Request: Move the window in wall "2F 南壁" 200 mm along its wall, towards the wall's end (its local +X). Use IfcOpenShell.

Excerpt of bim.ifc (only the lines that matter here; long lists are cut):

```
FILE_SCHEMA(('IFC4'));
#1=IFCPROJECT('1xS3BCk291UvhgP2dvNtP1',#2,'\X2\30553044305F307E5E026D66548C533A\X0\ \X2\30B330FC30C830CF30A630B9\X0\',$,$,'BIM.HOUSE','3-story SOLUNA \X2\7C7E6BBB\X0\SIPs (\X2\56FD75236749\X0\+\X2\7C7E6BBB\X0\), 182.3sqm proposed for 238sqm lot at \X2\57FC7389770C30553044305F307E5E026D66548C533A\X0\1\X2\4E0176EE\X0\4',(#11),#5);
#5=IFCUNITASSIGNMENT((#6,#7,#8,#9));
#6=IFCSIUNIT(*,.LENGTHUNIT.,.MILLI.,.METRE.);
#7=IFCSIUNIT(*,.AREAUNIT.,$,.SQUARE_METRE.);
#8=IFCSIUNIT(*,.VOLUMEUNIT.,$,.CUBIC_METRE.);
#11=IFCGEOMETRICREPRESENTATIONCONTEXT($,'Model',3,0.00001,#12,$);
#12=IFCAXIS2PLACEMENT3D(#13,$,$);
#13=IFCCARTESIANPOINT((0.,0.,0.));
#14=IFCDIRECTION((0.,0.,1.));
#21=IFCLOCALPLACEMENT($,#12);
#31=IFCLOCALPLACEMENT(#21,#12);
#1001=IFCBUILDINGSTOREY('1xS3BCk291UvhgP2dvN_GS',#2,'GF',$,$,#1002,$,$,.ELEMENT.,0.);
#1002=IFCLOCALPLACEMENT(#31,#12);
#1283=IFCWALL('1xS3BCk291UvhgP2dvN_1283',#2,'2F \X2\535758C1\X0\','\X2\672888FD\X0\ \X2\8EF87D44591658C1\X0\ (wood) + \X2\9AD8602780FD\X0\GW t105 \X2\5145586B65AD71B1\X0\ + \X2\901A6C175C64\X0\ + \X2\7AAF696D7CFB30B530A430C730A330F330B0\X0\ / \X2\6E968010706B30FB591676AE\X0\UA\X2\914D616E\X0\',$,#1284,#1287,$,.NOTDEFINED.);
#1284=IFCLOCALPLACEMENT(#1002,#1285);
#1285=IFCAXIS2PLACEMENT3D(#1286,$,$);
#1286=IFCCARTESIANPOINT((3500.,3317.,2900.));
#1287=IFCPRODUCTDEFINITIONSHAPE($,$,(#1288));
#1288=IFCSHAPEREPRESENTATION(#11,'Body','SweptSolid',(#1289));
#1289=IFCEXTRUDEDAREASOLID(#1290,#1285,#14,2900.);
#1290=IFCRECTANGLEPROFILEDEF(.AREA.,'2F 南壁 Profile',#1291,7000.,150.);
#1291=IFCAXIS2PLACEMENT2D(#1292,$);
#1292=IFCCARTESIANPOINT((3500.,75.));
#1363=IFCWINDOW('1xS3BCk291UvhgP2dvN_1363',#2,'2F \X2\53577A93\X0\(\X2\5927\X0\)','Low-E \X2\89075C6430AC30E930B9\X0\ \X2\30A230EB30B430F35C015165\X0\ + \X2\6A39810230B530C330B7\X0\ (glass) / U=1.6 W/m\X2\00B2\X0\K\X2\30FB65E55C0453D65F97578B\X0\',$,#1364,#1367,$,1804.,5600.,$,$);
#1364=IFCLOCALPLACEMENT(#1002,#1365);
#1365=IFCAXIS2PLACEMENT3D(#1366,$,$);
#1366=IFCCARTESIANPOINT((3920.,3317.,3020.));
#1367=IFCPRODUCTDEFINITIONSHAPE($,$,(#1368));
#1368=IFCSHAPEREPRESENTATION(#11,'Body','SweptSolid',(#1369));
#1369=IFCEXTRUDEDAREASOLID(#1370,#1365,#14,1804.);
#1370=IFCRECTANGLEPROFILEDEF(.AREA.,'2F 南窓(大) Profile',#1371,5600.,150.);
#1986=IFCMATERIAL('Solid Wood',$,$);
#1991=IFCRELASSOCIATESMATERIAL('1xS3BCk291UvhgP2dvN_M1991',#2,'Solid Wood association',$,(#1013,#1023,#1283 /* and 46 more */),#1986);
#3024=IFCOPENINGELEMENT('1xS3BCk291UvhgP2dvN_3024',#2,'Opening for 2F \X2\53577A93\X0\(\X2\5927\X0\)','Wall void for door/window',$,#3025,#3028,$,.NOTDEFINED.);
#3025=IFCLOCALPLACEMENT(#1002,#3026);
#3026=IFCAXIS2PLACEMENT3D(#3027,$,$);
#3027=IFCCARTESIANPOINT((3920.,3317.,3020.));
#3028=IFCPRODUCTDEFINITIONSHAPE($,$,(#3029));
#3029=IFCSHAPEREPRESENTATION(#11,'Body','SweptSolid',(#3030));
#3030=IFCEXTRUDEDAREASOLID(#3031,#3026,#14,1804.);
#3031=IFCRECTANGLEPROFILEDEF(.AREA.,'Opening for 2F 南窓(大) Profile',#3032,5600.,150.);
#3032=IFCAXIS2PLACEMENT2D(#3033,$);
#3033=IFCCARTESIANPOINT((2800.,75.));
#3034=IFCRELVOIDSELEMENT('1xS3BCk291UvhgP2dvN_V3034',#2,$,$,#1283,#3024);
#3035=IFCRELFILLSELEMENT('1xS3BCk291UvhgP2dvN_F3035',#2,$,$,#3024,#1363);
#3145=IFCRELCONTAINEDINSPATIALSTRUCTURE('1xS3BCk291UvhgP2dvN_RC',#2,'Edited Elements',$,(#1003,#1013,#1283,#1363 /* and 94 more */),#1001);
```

```python
import ifcopenshell
import ifcopenshell.api.geometry
import ifcopenshell.util.placement

model = ifcopenshell.open("bim.ifc")

window = model.by_id(1363)
opening = window.FillsVoids[0].RelatingOpeningElement
wall = opening.VoidsElements[0].RelatingBuildingElement

wall_matrix = ifcopenshell.util.placement.get_local_placement(wall.ObjectPlacement)
shift = wall_matrix[:3, 0] * 200.0
before = ifcopenshell.util.placement.get_local_placement(window.ObjectPlacement)[:3, 3].copy()

# The window is not placed relative to its opening, so move both.
for product in (opening, window):
    matrix = ifcopenshell.util.placement.get_local_placement(product.ObjectPlacement)
    matrix[:3, 3] += shift
    ifcopenshell.api.geometry.edit_object_placement(model, product=product, matrix=matrix, is_si=False)

after = ifcopenshell.util.placement.get_local_placement(window.ObjectPlacement)[:3, 3]
print("window moved by", (after - before).round(3) + 0.0)

model.write("bim_rev.ifc")
```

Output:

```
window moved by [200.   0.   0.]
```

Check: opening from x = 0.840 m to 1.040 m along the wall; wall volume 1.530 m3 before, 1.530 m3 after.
